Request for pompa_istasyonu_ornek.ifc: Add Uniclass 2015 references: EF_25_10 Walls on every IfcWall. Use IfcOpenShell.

First a look at what the model holds.

```python
import ifcopenshell

model = ifcopenshell.open("pompa_istasyonu_ornek.ifc")
print(model.schema)
print("classifications:", [c.Name for c in model.by_type("IfcClassification")])
for ifc_class in ("IfcDoor", "IfcRoof", "IfcStair", "IfcWall", "IfcWindow"):
    print(ifc_class, len(model.by_type(ifc_class)))
```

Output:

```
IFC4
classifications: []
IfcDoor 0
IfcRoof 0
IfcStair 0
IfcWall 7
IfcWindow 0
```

```python
import ifcopenshell
import ifcopenshell.api.classification

model = ifcopenshell.open("pompa_istasyonu_ornek.ifc")

system = ifcopenshell.api.classification.add_classification(model, classification="Uniclass 2015")

codes = {
    "IfcWall": ("EF_25_10", "Walls"),
}
for ifc_class, (code, name) in codes.items():
    products = model.by_type(ifc_class)
    ifcopenshell.api.classification.add_reference(
        model, products=products, classification=system, identification=code, name=name
    )
    print(code, len(products))

model.write("pompa_istasyonu_ornek_updated.ifc")
```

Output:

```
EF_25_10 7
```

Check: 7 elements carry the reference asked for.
